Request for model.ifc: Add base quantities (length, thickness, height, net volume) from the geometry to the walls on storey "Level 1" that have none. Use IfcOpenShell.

First a look at what the model holds.

```python
import ifcopenshell
import ifcopenshell.util.element
import ifcopenshell.util.unit

model = ifcopenshell.open("model.ifc")
print(model.schema)
for unit_type in ("LENGTHUNIT", "AREAUNIT", "VOLUMEUNIT"):
    print(unit_type, ifcopenshell.util.unit.calculate_unit_scale(model, unit_type))
storey = next(s for s in model.by_type("IfcBuildingStorey") if s.Name == "Level 1")
walls = [e for e in ifcopenshell.util.element.get_decomposition(storey) if e.is_a("IfcWall")]
for e in sorted(walls, key=lambda e: e.id()):
    print(e.id(), e.is_a(), e.Name, list(ifcopenshell.util.element.get_psets(e, qtos_only=True)), sep=" | ")
```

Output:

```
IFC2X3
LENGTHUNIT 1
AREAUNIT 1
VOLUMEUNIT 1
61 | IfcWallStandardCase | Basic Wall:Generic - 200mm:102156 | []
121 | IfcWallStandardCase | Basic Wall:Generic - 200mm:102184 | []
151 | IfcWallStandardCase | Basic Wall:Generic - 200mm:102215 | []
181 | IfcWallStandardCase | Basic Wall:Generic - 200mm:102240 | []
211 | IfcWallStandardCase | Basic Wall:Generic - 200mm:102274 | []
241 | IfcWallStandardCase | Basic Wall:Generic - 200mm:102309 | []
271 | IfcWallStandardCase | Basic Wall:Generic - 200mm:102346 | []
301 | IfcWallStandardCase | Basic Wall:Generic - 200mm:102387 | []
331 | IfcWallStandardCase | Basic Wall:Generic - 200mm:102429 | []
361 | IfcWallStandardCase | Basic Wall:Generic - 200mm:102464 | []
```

```python
import ifcopenshell
import ifcopenshell.api.pset
import ifcopenshell.geom
import ifcopenshell.util.element
import ifcopenshell.util.shape
import ifcopenshell.util.unit

model = ifcopenshell.open("model.ifc")
unit_scale = ifcopenshell.util.unit.calculate_unit_scale(model)
volume_scale = ifcopenshell.util.unit.calculate_unit_scale(model, "VOLUMEUNIT")
settings = ifcopenshell.geom.settings()

storey = next(s for s in model.by_type("IfcBuildingStorey") if s.Name == "Level 1")
walls = [e for e in ifcopenshell.util.element.get_decomposition(storey) if e.is_a("IfcWall")]

for e in sorted(walls, key=lambda e: e.id()):
    if ifcopenshell.util.element.get_psets(e, qtos_only=True, should_inherit=False):
        continue
    # Geometry comes back in metres, in the element's own axes.
    shape = ifcopenshell.geom.create_shape(settings, e)
    values = {
        "Length": ifcopenshell.util.shape.get_x(shape.geometry) / unit_scale,
        "Width": ifcopenshell.util.shape.get_y(shape.geometry) / unit_scale,
        "Height": ifcopenshell.util.shape.get_z(shape.geometry) / unit_scale,
        "NetVolume": ifcopenshell.util.shape.get_volume(shape.geometry) / volume_scale,
    }
    qto = ifcopenshell.api.pset.add_qto(model, product=e, name="BaseQuantities")
    ifcopenshell.api.pset.edit_qto(model, qto=qto, properties=values)
    print(e.id(), {k: round(v, 3) for k, v in values.items()})

model.write("model_edited.ifc")
```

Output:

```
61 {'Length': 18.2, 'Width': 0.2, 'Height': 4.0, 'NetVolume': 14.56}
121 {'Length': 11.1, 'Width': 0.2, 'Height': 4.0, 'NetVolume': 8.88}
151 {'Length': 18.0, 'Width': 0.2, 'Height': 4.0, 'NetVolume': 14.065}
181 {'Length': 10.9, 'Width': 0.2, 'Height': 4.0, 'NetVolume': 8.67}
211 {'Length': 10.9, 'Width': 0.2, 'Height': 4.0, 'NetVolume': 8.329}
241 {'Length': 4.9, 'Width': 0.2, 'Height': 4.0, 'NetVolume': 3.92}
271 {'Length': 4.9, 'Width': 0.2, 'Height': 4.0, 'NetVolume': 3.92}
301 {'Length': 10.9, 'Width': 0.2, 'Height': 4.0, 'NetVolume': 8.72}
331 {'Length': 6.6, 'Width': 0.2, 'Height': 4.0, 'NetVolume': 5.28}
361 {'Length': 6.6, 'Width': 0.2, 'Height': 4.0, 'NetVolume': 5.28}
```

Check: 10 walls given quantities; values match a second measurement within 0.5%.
